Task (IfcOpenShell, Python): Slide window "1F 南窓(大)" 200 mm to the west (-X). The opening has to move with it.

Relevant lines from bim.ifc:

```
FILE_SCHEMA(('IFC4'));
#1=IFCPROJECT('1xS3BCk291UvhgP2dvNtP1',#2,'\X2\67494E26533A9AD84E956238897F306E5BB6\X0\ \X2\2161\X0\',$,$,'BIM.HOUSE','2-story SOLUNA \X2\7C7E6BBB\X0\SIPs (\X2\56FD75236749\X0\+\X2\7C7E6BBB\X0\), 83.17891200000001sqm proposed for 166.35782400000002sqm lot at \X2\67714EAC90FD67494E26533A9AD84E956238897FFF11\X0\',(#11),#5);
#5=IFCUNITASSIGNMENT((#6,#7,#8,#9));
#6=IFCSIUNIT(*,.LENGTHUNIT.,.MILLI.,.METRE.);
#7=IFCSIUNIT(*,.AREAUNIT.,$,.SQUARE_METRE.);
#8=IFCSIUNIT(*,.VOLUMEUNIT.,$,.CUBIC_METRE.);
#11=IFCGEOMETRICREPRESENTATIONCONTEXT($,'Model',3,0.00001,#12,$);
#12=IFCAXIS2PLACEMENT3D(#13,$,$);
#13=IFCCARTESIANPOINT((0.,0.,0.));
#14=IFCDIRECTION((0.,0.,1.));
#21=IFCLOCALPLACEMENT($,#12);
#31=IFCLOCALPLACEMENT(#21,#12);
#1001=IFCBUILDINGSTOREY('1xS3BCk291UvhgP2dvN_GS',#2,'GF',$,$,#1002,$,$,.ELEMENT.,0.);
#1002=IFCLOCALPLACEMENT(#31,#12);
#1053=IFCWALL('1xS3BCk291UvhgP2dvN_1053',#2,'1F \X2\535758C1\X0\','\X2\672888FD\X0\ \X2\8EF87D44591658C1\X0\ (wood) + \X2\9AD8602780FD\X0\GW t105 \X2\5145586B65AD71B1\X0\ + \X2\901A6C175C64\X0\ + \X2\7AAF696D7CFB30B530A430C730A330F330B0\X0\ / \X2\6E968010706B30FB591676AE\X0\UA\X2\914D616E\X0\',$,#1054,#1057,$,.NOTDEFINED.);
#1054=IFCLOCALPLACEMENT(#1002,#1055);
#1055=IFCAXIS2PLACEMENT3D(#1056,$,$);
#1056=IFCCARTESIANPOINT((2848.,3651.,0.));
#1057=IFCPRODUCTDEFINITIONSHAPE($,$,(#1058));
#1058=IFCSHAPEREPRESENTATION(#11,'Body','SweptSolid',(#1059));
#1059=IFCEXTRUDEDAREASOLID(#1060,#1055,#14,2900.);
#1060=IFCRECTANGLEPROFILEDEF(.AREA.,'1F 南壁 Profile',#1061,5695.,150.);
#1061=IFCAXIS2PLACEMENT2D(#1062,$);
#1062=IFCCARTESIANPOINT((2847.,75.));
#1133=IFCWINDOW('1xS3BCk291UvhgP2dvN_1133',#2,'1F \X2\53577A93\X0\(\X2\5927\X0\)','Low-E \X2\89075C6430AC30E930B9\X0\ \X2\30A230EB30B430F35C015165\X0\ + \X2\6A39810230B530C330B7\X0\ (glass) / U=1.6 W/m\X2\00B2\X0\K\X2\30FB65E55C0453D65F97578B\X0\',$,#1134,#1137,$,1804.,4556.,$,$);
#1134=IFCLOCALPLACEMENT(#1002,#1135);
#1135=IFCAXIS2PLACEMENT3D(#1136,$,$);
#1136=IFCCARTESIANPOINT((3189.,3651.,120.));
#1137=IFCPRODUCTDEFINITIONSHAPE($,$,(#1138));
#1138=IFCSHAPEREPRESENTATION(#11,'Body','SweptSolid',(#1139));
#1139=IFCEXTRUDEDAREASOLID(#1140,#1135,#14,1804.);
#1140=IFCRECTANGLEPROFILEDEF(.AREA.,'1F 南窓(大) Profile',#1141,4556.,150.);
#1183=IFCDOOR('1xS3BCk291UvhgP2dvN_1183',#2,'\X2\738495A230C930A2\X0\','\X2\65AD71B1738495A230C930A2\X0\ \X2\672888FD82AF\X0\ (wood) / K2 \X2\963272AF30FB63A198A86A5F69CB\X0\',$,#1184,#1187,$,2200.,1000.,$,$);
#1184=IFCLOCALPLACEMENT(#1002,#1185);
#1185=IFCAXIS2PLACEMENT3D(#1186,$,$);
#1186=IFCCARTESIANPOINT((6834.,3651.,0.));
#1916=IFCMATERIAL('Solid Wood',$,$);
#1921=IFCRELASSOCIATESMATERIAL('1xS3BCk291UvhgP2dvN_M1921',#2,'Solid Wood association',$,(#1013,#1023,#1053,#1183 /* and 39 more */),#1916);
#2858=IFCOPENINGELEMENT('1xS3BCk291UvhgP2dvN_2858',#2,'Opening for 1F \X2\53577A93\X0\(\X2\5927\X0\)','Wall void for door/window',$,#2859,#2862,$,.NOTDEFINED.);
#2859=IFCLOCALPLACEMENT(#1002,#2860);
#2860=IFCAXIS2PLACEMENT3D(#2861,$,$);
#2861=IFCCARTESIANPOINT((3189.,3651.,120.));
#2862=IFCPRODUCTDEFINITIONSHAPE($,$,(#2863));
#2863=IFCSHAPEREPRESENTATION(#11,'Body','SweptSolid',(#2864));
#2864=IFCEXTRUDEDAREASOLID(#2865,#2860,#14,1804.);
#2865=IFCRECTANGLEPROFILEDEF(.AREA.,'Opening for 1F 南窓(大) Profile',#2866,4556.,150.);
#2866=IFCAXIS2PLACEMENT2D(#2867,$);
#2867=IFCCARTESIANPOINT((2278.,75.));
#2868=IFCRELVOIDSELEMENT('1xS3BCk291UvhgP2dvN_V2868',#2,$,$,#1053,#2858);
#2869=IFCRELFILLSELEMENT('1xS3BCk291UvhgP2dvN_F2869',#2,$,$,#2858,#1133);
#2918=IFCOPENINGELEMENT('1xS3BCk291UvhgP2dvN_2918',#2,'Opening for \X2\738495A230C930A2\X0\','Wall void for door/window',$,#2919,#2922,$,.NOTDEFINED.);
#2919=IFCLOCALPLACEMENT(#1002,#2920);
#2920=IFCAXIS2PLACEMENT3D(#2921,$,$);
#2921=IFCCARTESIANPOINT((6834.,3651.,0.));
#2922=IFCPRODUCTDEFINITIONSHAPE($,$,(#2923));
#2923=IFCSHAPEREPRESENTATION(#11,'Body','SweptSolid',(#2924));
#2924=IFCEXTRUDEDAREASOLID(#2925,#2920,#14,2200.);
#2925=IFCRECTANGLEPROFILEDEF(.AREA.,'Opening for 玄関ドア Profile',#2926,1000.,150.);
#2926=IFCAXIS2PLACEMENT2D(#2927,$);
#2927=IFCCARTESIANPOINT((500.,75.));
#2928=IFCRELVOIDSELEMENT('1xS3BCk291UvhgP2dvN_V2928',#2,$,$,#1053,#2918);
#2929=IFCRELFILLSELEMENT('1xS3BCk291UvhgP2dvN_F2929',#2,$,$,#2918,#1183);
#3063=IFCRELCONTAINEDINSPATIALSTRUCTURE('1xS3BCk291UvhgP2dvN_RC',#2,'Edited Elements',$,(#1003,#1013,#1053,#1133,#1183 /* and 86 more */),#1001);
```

```python
import ifcopenshell
import ifcopenshell.api.geometry
import ifcopenshell.util.placement
import ifcopenshell.util.unit

model = ifcopenshell.open("bim.ifc")
unit_scale = ifcopenshell.util.unit.calculate_unit_scale(model)

window = model.by_guid("1xS3BCk291UvhgP2dvN_1133")
opening = window.FillsVoids[0].RelatingOpeningElement
wall = opening.VoidsElements[0].RelatingBuildingElement

wall_matrix = ifcopenshell.util.placement.get_local_placement(wall.ObjectPlacement)
shift = wall_matrix[:3, 0] * -0.2 / unit_scale
before = ifcopenshell.util.placement.get_local_placement(window.ObjectPlacement)[:3, 3].copy()

# The window is not placed relative to its opening, so move both.
for product in (opening, window):
    matrix = ifcopenshell.util.placement.get_local_placement(product.ObjectPlacement)
    matrix[:3, 3] += shift
    ifcopenshell.api.geometry.edit_object_placement(model, product=product, matrix=matrix, is_si=False)

after = ifcopenshell.util.placement.get_local_placement(window.ObjectPlacement)[:3, 3]
print("window moved by", (after - before).round(3) + 0.0)

model.write("bim_rev.ifc")
```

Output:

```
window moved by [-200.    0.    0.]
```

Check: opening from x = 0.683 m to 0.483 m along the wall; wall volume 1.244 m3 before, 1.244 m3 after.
